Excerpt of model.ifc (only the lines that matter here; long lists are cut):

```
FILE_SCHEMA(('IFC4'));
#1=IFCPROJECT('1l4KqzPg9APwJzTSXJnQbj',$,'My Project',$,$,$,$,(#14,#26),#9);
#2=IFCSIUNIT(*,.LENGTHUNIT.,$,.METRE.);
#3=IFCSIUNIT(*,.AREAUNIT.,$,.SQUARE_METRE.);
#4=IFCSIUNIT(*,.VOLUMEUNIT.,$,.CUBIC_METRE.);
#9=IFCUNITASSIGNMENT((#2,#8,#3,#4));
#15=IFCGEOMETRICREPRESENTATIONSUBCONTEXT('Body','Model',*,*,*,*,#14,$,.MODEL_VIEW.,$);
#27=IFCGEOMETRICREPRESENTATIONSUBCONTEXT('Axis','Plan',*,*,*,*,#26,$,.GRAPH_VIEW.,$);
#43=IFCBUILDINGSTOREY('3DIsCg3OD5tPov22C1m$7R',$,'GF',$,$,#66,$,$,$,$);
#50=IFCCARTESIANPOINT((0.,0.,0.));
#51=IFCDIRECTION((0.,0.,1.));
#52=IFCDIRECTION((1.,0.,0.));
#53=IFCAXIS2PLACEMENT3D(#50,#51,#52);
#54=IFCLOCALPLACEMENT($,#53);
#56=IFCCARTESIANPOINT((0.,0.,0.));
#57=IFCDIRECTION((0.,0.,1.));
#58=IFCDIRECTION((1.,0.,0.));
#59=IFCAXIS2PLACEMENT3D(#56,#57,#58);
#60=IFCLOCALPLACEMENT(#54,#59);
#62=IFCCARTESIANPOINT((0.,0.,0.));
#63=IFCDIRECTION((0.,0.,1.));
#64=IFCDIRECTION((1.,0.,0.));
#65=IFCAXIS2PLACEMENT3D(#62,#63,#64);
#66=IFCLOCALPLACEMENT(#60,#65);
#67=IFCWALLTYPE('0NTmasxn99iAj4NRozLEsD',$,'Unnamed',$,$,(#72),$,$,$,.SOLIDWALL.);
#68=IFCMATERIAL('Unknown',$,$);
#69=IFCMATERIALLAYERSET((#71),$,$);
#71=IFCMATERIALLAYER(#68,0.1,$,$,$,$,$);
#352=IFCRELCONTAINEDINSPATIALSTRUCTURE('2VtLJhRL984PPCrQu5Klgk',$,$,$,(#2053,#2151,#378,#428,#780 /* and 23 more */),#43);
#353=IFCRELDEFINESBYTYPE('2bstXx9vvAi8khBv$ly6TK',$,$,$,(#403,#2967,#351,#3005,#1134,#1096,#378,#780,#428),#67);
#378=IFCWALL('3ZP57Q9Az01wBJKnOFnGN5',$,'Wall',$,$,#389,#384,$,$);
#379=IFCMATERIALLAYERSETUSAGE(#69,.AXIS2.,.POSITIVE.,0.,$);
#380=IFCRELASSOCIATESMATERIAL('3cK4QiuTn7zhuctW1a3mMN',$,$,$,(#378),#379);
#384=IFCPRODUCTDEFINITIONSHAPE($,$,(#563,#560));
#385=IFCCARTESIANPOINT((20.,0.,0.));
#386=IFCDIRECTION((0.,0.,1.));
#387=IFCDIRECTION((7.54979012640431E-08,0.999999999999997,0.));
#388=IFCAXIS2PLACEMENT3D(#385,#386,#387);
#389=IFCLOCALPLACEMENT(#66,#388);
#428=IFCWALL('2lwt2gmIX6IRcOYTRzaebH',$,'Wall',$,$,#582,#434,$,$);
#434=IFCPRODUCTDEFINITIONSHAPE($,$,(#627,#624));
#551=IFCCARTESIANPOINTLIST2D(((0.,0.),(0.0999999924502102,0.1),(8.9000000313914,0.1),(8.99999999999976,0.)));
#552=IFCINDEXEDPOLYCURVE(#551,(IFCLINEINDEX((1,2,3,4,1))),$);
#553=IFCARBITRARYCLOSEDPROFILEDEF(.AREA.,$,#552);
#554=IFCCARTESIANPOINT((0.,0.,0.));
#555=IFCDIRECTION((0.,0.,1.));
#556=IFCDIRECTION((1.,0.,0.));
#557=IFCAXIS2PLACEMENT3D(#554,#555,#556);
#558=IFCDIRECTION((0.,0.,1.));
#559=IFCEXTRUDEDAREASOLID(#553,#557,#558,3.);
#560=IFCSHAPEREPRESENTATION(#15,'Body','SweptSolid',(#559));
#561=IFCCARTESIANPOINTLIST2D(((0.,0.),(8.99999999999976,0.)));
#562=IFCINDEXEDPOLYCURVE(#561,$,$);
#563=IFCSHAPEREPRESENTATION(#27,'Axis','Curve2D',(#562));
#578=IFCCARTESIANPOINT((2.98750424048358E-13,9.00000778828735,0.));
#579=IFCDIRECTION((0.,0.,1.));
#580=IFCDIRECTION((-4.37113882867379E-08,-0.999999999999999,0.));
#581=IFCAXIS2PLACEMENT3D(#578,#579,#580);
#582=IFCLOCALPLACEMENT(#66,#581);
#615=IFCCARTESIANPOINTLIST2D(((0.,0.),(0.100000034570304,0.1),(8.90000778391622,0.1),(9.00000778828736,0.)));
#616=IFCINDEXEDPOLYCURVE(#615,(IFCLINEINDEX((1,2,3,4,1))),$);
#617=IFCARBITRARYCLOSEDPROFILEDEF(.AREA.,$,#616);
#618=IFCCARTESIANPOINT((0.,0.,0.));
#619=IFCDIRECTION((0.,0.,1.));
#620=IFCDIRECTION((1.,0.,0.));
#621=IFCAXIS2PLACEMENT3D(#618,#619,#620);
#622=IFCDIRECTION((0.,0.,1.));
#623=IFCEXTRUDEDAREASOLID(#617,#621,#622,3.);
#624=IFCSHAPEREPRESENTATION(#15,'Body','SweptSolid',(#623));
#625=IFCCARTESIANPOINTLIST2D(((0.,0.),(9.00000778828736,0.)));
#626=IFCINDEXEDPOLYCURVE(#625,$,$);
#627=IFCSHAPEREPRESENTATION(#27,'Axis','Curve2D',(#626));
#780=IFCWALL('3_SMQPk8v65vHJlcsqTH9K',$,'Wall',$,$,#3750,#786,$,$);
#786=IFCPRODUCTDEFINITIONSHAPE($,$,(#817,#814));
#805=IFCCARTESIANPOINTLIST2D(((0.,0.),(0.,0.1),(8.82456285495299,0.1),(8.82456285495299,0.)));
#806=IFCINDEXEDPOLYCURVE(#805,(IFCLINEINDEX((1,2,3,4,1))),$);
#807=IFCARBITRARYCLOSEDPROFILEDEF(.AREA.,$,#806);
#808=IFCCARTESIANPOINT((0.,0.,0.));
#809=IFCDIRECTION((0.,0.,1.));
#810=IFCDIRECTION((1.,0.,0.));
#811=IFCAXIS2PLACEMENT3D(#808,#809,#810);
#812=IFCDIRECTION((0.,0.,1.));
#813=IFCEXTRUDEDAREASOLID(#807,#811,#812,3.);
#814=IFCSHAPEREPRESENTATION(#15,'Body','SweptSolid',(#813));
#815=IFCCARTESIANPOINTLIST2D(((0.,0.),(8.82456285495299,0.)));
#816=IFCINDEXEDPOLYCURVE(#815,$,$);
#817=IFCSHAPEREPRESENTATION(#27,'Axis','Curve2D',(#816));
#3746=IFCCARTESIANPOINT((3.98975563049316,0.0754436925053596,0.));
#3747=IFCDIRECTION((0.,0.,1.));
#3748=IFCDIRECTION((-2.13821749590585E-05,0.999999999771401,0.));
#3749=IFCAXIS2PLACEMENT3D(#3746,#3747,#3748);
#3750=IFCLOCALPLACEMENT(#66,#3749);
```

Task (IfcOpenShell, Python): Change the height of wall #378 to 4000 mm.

```python
import ifcopenshell
import ifcopenshell.geom
import ifcopenshell.util.representation
import ifcopenshell.util.shape

model = ifcopenshell.open("model.ifc")
settings = ifcopenshell.geom.settings()


def volume(element):
    """Net volume in cubic metres, openings subtracted."""
    shape = ifcopenshell.geom.create_shape(settings, element)
    return ifcopenshell.util.shape.get_volume(shape.geometry)


wall = model.by_guid("3ZP57Q9Az01wBJKnOFnGN5")
before = volume(wall)

body = ifcopenshell.util.representation.get_representation(wall, "Model", "Body")
solid = body.Items[0]
old_height = solid.Depth
solid.Depth = 4.0
after = volume(wall)

print(f"height {old_height:g} -> {solid.Depth:g}, volume {before:.3f} -> {after:.3f} m3")

model.write("model_edited.ifc")
```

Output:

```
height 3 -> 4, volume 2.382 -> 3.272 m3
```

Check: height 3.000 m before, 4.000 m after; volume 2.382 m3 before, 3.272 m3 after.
